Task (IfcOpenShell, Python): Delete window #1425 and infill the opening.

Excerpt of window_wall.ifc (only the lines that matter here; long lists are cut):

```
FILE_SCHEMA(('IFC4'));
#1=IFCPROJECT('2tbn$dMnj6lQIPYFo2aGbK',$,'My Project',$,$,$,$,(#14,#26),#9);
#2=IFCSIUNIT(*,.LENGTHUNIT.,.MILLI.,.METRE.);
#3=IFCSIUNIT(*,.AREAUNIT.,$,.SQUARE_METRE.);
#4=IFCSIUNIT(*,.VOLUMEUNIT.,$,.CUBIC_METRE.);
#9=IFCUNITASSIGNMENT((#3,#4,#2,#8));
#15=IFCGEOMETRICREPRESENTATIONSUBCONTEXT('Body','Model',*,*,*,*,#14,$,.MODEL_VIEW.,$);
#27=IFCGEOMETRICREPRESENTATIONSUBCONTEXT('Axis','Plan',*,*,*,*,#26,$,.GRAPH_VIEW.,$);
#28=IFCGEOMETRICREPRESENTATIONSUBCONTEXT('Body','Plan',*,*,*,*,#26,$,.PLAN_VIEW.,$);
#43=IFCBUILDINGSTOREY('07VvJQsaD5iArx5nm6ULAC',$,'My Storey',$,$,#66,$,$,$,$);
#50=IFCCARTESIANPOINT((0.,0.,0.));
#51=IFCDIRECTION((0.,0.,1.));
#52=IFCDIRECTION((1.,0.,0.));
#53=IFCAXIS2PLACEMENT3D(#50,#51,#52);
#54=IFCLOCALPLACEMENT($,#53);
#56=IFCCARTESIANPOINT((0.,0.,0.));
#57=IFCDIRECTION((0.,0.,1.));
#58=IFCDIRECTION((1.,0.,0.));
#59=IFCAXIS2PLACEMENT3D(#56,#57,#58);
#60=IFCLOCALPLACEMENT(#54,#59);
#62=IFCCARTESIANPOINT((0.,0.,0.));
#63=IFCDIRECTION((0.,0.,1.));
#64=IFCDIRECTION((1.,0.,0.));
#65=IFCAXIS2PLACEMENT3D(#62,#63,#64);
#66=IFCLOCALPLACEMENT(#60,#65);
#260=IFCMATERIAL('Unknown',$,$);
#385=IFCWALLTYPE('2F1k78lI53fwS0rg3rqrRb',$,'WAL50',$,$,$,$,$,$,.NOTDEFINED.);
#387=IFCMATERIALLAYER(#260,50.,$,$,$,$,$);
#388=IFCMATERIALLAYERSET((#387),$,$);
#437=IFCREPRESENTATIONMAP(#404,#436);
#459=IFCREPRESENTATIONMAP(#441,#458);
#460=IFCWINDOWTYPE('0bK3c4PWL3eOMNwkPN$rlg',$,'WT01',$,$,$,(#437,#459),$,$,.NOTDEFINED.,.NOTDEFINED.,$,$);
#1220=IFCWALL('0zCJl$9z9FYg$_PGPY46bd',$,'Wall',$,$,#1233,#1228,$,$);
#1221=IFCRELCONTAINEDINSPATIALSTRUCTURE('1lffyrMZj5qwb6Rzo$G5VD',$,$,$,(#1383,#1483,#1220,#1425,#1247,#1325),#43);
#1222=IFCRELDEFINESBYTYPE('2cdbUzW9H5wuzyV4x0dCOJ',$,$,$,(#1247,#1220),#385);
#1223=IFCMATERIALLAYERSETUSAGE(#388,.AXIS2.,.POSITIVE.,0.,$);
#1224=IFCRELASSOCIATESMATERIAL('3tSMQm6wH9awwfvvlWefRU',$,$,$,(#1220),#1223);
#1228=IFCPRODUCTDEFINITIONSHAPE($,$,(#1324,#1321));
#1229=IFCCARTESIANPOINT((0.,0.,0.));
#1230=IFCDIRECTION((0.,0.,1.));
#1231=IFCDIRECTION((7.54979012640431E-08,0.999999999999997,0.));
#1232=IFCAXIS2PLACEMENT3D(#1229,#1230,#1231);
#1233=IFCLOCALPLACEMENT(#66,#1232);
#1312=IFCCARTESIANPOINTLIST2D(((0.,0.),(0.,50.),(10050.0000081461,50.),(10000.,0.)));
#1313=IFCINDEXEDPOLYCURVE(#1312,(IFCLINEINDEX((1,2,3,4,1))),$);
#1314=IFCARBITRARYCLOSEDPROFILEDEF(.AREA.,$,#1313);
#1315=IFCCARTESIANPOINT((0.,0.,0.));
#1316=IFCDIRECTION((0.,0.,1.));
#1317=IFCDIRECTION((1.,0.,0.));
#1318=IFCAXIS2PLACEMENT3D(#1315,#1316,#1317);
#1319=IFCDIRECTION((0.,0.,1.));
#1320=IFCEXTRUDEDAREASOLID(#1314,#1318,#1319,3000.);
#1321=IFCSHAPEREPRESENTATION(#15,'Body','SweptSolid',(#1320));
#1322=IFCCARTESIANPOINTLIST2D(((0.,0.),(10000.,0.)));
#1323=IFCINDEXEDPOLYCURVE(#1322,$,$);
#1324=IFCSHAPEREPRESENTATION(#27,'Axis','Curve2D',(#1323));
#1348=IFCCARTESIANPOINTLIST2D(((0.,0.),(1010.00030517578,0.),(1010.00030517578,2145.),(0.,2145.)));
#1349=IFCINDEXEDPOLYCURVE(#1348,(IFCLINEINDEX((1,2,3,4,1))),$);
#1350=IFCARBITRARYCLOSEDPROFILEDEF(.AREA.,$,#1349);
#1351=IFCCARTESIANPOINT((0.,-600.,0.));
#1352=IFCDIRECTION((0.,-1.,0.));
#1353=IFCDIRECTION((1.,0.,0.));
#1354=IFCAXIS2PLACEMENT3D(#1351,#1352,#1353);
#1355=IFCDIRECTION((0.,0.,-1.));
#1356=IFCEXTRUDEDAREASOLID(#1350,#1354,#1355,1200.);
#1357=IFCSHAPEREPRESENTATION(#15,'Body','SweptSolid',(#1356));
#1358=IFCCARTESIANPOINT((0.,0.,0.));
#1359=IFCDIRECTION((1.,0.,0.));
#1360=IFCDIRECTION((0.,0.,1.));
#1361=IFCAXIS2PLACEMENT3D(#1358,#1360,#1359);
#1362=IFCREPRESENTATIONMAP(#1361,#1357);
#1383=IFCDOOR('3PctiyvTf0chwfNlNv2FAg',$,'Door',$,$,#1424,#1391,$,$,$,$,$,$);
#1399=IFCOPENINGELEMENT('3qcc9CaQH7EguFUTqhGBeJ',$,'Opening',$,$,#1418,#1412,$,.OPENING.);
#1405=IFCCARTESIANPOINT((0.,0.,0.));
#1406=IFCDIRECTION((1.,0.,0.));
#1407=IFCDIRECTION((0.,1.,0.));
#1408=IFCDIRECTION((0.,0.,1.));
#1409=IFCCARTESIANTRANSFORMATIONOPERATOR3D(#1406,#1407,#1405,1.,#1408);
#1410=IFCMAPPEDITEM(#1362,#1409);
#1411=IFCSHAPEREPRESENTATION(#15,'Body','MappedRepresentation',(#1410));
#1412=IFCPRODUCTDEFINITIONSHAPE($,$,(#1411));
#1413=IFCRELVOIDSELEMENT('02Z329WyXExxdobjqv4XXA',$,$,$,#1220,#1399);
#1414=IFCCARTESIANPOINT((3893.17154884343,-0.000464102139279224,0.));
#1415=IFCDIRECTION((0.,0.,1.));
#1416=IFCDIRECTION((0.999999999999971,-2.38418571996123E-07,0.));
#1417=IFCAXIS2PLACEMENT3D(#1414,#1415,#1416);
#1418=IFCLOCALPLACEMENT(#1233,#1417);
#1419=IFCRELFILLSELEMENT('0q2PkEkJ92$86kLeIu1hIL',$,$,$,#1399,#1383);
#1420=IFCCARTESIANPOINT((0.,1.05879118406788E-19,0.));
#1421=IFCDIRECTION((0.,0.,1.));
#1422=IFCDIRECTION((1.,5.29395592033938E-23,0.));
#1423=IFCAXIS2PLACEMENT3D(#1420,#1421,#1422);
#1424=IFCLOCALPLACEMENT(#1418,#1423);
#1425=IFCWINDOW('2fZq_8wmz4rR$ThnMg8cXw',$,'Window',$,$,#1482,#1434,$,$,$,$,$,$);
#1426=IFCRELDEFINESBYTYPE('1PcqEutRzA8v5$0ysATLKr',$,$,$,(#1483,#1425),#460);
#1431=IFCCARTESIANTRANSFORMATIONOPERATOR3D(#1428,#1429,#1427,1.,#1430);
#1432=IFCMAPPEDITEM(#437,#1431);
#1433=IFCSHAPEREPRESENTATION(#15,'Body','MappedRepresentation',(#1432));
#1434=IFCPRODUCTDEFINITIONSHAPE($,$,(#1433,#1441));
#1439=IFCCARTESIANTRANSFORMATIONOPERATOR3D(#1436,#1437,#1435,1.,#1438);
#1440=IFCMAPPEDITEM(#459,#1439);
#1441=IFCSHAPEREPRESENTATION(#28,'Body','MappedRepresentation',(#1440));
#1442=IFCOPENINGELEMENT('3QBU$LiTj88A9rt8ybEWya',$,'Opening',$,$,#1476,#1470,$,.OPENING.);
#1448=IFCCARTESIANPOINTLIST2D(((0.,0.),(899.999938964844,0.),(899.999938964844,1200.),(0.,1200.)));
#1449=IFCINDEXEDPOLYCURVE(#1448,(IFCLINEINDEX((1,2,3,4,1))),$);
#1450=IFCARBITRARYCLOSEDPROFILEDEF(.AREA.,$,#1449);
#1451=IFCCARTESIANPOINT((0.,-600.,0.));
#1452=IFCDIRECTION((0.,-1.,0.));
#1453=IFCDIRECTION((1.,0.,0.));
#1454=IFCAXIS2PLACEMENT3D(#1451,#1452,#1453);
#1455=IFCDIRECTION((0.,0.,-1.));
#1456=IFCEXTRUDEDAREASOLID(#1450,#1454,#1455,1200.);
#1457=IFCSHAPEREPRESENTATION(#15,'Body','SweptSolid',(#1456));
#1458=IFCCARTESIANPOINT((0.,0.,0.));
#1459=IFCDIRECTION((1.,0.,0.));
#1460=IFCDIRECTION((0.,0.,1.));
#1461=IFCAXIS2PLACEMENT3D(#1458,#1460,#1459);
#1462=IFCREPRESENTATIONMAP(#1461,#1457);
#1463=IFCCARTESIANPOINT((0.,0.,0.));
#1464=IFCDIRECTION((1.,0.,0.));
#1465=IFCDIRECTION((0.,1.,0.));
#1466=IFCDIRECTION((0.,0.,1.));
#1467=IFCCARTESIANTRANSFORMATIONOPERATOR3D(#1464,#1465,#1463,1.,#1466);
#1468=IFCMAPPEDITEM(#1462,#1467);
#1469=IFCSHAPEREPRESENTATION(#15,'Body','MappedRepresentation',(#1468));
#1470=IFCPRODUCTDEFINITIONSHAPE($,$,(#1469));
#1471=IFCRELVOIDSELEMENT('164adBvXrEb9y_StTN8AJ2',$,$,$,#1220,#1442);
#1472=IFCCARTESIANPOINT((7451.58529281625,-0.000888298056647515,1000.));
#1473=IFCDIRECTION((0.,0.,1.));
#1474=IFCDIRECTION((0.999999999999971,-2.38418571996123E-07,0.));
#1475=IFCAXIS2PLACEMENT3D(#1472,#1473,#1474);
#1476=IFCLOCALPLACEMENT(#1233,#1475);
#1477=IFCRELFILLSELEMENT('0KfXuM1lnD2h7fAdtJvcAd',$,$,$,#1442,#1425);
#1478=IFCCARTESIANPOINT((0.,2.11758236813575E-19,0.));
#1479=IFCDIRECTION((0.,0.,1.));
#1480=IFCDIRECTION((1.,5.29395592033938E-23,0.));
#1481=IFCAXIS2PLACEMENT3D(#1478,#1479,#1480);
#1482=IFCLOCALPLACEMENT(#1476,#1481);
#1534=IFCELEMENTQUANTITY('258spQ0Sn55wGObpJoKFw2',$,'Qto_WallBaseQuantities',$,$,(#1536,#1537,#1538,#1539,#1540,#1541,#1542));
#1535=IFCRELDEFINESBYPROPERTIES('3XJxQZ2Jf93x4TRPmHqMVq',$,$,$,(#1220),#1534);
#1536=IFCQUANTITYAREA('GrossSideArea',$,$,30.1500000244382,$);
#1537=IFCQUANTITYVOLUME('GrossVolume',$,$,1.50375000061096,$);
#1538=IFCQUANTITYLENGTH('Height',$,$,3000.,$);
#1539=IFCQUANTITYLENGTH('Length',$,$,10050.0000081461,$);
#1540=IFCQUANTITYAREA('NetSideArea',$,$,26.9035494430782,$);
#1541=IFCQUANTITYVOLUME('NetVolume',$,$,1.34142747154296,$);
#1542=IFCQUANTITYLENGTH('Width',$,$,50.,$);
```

```python
import ifcopenshell
import ifcopenshell.api.feature
import ifcopenshell.api.pset
import ifcopenshell.api.root
import ifcopenshell.geom
import ifcopenshell.util.element
import ifcopenshell.util.shape
import ifcopenshell.util.unit

model = ifcopenshell.open("window_wall.ifc")
area_scale = ifcopenshell.util.unit.calculate_unit_scale(model, "AREAUNIT")
volume_scale = ifcopenshell.util.unit.calculate_unit_scale(model, "VOLUMEUNIT")
settings = ifcopenshell.geom.settings()


def volume(element):
    """Net volume in cubic metres, openings subtracted."""
    shape = ifcopenshell.geom.create_shape(settings, element)
    return ifcopenshell.util.shape.get_volume(shape.geometry)


window = model.by_guid("2fZq_8wmz4rR$ThnMg8cXw")
opening = window.FillsVoids[0].RelatingOpeningElement
wall = opening.VoidsElements[0].RelatingBuildingElement
before = volume(wall)

ifcopenshell.api.root.remove_product(model, product=window)
ifcopenshell.api.feature.remove_feature(model, feature=opening)

after = volume(wall)
thickness = 0.05  # wall thickness in metres

# Update the wall's stored quantities.
qto = model.by_id(ifcopenshell.util.element.get_pset(wall, "Qto_WallBaseQuantities", should_inherit=False)["id"])
ifcopenshell.api.pset.edit_qto(model, qto=qto, properties={
    "NetSideArea": after / thickness / area_scale,
    "NetVolume": after / volume_scale,
})

print(f"wall volume {before:.3f} -> {after:.3f} m3")

model.write("window_wall-out.ifc")
```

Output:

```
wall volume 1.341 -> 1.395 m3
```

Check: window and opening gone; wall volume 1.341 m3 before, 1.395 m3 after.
